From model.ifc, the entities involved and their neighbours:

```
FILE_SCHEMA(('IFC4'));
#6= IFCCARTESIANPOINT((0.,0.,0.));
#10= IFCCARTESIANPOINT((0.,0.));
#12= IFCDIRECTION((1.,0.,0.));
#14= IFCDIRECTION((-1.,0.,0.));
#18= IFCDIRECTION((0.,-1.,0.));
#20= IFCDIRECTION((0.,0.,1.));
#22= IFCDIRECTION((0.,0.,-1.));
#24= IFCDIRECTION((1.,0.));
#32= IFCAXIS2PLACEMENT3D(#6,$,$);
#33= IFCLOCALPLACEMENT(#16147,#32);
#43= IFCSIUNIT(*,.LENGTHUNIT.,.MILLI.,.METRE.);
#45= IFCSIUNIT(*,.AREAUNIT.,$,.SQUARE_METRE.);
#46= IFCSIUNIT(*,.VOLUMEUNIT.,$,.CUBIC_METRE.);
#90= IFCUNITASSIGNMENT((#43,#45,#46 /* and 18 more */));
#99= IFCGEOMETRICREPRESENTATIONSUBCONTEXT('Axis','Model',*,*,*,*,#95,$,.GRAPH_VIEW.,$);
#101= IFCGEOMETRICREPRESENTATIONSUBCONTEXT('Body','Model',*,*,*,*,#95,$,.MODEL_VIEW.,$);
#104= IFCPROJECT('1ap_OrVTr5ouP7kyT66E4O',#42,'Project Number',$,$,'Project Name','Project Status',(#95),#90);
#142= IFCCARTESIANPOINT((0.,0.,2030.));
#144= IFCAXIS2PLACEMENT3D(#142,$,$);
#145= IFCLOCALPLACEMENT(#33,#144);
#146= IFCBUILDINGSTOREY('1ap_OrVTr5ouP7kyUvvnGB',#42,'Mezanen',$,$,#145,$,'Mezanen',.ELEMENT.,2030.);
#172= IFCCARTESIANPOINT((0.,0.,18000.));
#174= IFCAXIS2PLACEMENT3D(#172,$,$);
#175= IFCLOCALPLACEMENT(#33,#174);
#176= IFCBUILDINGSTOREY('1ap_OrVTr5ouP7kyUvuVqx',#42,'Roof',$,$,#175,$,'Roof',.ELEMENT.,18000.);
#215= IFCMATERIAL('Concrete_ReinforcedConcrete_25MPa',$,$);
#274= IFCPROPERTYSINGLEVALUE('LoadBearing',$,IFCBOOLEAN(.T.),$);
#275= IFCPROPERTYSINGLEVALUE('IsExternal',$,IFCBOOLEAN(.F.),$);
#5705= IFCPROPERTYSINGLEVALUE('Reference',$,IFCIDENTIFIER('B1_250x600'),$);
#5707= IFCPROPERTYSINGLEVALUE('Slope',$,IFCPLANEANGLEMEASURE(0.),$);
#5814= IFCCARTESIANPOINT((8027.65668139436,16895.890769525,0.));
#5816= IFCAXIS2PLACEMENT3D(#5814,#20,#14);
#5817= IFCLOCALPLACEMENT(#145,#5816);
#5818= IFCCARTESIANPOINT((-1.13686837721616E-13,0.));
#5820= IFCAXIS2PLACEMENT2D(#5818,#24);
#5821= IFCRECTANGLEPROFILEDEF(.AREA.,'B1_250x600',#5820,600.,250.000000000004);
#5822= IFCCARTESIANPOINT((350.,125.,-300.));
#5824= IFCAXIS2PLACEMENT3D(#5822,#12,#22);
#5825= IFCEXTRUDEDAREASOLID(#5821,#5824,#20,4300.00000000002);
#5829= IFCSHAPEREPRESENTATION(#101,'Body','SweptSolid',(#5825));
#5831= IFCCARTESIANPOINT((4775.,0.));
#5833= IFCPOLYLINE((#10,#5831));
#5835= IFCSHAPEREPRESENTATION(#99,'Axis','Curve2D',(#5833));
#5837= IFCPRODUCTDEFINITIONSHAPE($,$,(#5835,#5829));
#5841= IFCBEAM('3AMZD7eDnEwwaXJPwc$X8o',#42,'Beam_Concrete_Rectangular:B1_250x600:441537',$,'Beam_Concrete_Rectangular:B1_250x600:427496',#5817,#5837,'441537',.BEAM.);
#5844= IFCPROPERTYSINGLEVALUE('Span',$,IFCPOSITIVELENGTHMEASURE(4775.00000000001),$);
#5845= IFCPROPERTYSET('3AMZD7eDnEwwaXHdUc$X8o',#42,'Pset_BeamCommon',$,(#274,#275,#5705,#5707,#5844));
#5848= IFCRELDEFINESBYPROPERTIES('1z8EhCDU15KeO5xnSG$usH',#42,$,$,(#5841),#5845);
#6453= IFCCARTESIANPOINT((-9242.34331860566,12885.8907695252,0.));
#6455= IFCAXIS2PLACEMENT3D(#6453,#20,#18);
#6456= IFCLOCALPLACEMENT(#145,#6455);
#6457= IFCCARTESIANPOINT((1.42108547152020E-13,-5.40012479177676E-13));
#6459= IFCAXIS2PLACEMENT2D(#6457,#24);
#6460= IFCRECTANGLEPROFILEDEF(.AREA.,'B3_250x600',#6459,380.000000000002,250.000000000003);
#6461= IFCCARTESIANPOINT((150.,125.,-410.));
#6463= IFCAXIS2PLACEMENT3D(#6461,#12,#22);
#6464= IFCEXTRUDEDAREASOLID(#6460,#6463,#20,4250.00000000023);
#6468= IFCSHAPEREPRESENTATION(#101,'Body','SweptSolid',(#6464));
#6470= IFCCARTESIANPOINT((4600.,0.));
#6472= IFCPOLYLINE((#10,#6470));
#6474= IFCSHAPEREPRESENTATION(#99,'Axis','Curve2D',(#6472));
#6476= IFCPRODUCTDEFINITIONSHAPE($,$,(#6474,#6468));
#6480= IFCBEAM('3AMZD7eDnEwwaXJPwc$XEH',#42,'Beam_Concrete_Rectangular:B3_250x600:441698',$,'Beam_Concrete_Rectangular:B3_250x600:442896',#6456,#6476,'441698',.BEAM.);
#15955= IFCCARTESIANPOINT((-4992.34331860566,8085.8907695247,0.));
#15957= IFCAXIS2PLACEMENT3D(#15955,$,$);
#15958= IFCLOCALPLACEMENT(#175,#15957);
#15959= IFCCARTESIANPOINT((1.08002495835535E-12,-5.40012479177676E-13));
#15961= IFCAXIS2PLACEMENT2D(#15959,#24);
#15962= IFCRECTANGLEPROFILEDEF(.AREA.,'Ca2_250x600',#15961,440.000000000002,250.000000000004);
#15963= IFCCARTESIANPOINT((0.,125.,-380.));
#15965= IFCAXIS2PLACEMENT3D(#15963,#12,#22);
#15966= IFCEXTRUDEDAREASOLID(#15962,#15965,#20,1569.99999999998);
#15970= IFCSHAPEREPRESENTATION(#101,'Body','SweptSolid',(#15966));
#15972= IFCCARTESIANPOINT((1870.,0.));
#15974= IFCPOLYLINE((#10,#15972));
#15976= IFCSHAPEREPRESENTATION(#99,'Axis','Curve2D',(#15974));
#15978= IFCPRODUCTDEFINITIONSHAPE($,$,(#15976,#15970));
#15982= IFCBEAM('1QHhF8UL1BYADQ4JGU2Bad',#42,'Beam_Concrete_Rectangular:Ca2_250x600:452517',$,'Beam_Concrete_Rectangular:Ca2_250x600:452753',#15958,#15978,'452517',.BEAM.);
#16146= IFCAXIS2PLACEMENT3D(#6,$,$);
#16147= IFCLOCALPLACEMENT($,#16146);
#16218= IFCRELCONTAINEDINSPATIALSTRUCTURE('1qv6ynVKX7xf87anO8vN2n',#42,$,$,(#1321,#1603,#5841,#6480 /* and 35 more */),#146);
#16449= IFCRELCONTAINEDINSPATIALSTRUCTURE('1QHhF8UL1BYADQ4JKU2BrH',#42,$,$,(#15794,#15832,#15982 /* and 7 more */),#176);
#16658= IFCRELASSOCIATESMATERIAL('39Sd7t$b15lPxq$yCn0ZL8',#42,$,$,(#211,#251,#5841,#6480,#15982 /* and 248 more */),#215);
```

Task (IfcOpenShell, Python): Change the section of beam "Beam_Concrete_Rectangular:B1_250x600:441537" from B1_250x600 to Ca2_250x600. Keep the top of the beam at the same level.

```python
import ifcopenshell
import ifcopenshell.api.pset
import ifcopenshell.util.element
import ifcopenshell.util.representation

model = ifcopenshell.open("model.ifc")

member = model.by_guid("3AMZD7eDnEwwaXJPwc$X8o")
source = next(p for p in model.by_type("IfcRectangleProfileDef") if p.ProfileName == "Ca2_250x600")

body = ifcopenshell.util.representation.get_representation(member, "Model", "Body")
solid = body.Items[0]
old_profile = solid.SweptArea

# Copy the section's sizes but keep this member's own profile position.
profile = ifcopenshell.util.element.copy(model, source)
# Profiles are centred, so shift by half the change in depth to hold the top.
shift = (old_profile.XDim - profile.XDim) / 2
x, y = old_profile.Position.Location.Coordinates
up = (-1.0, 0.0)  # upwards, in the solid's own plane
location = model.createIfcCartesianPoint((x + up[0] * shift, y + up[1] * shift))
profile.Position = model.createIfcAxis2Placement2D(location, old_profile.Position.RefDirection)
solid.SweptArea = profile
if not model.get_total_inverses(old_profile):
    ifcopenshell.util.element.remove_deep2(model, old_profile)
member.Name = member.Name.replace("B1_250x600", "Ca2_250x600")
member.ObjectType = member.ObjectType.replace("B1_250x600", "Ca2_250x600")
pset = model.by_id(ifcopenshell.util.element.get_pset(member, "Pset_BeamCommon", should_inherit=False)["id"])
ifcopenshell.api.pset.edit_pset(model, pset=pset, properties={"Reference": "Ca2_250x600"})

print(solid.SweptArea)

model.write("model_updated.ifc")
```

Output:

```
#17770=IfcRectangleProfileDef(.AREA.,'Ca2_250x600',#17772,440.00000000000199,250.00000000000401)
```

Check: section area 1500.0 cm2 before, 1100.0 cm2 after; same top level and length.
